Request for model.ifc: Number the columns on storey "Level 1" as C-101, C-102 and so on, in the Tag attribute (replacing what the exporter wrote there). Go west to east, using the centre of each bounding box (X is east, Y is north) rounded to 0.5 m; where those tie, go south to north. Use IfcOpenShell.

First a look at what the model holds.

```python
import ifcopenshell
import ifcopenshell.util.element
import ifcopenshell.util.placement

model = ifcopenshell.open("model.ifc")
print(model.schema)
storey = next(s for s in model.by_type("IfcBuildingStorey") if s.Name == "Level 1")
columns = [e for e in ifcopenshell.util.element.get_decomposition(storey) if e.is_a("IfcColumn")]
for e in sorted(columns, key=lambda e: e.id()):
    origin = ifcopenshell.util.placement.get_local_placement(e.ObjectPlacement)[:3, 3]
    print(e.id(), e.Tag, e.Name, origin.round(2) + 0.0, sep=" | ")
```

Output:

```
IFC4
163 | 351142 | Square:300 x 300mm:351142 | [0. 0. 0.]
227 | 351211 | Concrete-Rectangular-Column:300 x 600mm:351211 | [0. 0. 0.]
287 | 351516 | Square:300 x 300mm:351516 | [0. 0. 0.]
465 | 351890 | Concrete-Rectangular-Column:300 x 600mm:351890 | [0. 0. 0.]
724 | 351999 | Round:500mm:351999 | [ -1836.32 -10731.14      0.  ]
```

```python
import ifcopenshell
import ifcopenshell.geom
import ifcopenshell.util.element
import ifcopenshell.util.shape

model = ifcopenshell.open("model.ifc")
settings = ifcopenshell.geom.settings()
settings.set("use-world-coords", True)


def centre(element):
    shape = ifcopenshell.geom.create_shape(settings, element)
    return ifcopenshell.util.shape.get_bbox_centroid(shape.geometry)


storey = next(s for s in model.by_type("IfcBuildingStorey") if s.Name == "Level 1")
columns = [e for e in ifcopenshell.util.element.get_decomposition(storey) if e.is_a("IfcColumn")]

# Insertion points can sit at a corner or the storey origin, so sort by the geometry (in metres).
centres = {e: centre(e) for e in columns}
columns.sort(key=lambda e: (round(centres[e][0] / 0.5), centres[e][1]))

for i, e in enumerate(columns, start=1):
    number = f"C-1{i:02d}"
    e.Tag = number
    print(e.id(), number)

model.write("model_rev.ifc")
```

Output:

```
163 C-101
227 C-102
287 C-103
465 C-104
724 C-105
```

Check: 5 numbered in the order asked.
